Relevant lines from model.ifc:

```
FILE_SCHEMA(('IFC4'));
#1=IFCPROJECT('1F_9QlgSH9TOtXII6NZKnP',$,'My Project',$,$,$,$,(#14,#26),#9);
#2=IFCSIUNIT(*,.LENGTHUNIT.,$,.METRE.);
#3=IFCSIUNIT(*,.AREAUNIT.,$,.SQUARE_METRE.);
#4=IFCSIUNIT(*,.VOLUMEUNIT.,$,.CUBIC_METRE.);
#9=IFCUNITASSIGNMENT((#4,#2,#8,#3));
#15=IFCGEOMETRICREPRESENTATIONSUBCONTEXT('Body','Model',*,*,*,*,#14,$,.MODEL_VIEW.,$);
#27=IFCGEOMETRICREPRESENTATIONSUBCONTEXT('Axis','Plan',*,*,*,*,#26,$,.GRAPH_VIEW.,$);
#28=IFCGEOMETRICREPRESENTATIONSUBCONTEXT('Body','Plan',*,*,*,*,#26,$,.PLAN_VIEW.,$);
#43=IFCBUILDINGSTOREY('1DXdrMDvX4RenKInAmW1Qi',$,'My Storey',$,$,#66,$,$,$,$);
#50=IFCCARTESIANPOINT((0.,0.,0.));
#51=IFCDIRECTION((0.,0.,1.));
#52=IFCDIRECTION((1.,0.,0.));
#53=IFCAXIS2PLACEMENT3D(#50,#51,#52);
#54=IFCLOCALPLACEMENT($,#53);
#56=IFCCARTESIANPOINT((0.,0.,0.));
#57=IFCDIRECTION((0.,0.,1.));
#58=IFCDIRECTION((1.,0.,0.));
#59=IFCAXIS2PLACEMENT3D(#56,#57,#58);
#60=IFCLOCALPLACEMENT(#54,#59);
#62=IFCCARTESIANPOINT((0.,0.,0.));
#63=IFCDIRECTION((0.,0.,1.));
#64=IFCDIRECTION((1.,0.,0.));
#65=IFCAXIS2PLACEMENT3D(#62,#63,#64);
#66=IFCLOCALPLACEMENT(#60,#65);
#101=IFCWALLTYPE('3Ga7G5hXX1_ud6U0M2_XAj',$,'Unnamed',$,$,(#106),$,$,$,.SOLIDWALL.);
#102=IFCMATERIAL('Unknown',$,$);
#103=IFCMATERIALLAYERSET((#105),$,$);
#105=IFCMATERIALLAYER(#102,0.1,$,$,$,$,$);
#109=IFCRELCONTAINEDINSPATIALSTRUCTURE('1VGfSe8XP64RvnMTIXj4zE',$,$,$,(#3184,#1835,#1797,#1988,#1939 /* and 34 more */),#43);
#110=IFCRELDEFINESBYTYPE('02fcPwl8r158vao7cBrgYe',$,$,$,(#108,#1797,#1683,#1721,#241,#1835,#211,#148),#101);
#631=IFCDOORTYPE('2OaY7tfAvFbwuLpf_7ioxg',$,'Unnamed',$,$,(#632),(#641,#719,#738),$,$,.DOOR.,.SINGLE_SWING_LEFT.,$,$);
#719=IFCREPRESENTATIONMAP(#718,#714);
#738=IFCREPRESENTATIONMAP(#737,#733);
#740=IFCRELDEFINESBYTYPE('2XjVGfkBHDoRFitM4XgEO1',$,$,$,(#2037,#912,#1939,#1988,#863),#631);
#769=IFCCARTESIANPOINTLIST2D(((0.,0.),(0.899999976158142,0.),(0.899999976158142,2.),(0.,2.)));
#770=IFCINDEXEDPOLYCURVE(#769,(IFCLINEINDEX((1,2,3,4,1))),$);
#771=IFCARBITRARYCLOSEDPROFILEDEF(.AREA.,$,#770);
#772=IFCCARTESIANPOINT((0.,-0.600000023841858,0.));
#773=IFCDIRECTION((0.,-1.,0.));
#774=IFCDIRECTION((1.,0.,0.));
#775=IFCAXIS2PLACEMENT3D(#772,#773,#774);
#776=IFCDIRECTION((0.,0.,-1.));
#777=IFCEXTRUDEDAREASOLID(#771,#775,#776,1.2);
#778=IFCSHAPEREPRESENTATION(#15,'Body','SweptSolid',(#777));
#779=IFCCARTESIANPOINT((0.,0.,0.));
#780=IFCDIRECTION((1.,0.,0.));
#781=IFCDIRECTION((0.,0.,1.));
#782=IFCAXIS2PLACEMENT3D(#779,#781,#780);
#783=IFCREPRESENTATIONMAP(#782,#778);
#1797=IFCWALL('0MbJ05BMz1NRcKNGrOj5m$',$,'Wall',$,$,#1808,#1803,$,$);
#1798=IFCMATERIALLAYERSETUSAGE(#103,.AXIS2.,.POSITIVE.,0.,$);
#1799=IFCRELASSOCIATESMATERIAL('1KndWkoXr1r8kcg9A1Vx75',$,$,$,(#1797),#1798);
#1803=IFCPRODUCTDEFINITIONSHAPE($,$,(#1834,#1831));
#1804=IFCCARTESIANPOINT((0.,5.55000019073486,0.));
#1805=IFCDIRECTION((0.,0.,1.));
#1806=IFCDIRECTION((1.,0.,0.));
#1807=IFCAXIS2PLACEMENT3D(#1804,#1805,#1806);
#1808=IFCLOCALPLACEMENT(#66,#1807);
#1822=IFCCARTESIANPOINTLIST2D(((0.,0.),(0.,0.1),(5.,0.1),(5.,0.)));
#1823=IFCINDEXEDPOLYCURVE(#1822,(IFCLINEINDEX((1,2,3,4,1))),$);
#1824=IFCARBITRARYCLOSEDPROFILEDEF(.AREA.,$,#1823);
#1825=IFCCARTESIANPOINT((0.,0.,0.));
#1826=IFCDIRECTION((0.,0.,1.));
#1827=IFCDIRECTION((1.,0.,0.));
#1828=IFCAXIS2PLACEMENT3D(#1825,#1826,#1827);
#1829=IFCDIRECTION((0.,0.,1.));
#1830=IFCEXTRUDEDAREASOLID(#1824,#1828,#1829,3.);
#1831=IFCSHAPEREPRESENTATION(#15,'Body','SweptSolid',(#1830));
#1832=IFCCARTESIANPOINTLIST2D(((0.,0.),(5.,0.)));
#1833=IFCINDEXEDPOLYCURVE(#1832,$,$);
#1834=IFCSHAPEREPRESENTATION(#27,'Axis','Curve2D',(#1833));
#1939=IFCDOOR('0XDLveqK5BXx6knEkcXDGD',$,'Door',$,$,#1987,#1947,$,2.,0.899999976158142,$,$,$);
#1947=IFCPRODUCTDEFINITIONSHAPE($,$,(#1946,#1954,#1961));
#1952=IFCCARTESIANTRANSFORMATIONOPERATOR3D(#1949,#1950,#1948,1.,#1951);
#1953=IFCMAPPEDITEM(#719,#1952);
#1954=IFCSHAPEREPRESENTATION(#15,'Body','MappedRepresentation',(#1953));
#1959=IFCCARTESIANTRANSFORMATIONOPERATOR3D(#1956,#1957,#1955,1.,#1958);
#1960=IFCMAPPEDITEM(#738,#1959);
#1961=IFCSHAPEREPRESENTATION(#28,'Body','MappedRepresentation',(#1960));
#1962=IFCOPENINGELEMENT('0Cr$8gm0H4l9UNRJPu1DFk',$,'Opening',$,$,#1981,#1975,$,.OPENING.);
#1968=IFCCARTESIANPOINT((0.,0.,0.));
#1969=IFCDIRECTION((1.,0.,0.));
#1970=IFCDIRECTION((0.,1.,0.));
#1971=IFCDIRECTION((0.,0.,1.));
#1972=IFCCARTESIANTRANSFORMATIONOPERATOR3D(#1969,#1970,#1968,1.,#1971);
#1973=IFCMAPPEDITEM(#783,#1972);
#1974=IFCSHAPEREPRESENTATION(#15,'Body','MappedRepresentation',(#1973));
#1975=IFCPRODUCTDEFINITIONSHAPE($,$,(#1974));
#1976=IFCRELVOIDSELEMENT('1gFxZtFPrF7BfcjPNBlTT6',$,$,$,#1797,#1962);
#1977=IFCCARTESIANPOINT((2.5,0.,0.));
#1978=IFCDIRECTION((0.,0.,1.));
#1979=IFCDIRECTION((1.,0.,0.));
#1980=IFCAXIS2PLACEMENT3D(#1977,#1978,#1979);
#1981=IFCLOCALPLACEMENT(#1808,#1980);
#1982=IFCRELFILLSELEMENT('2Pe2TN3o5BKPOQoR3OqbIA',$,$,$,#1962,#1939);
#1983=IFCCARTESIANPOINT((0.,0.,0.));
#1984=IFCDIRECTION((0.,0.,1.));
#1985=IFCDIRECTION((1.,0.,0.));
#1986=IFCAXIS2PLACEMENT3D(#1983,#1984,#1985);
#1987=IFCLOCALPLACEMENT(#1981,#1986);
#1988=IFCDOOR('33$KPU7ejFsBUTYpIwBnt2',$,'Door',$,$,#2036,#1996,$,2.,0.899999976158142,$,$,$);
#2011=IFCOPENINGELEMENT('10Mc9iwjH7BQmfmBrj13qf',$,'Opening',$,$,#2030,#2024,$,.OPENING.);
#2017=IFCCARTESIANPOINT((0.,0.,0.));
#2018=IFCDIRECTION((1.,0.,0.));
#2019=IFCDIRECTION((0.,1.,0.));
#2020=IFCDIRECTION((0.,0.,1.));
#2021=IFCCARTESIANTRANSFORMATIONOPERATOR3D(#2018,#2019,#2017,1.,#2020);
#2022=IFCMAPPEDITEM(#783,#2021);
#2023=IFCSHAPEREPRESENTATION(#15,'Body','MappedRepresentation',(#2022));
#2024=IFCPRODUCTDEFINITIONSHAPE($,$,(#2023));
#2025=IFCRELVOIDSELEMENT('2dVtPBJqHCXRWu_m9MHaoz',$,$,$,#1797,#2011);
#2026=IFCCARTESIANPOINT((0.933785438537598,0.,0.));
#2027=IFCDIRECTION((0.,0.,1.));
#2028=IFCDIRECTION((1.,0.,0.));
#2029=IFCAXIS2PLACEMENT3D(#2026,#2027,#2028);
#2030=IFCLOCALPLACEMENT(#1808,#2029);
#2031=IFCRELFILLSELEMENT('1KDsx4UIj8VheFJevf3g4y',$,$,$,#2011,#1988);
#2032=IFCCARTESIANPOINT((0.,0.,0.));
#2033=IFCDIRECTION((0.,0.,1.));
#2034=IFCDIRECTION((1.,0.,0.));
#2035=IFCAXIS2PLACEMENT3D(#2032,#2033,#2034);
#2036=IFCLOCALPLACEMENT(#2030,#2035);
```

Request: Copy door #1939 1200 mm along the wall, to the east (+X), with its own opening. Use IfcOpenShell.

```python
import ifcopenshell
import ifcopenshell.api.feature
import ifcopenshell.api.geometry
import ifcopenshell.api.root
import ifcopenshell.geom
import ifcopenshell.util.element
import ifcopenshell.util.placement
import ifcopenshell.util.shape
import ifcopenshell.util.unit

model = ifcopenshell.open("model.ifc")
unit_scale = ifcopenshell.util.unit.calculate_unit_scale(model)
settings = ifcopenshell.geom.settings()


def volume(element):
    """Net volume in cubic metres, openings subtracted."""
    shape = ifcopenshell.geom.create_shape(settings, element)
    return ifcopenshell.util.shape.get_volume(shape.geometry)


door = model.by_guid("0XDLveqK5BXx6knEkcXDGD")
opening = door.FillsVoids[0].RelatingOpeningElement
wall = opening.VoidsElements[0].RelatingBuildingElement
before = volume(wall)
shift = ifcopenshell.util.placement.get_local_placement(wall.ObjectPlacement)[:3, 0] * 1.2 / unit_scale

# copy_class copies the void relationship, type, container and properties, but no geometry.
new_opening = ifcopenshell.api.root.copy_class(model, product=opening)
new_opening.Representation = ifcopenshell.util.element.copy_deep(
    model, opening.Representation, exclude=["IfcGeometricRepresentationContext", "IfcRepresentationMap"]
)
new_door = ifcopenshell.api.root.copy_class(model, product=door)
new_door.Representation = ifcopenshell.util.element.copy_deep(
    model, door.Representation, exclude=["IfcGeometricRepresentationContext", "IfcRepresentationMap"]
)
ifcopenshell.api.feature.add_filling(model, opening=new_opening, element=new_door)

for old, new in ((opening, new_opening), (door, new_door)):
    matrix = ifcopenshell.util.placement.get_local_placement(old.ObjectPlacement)
    matrix[:3, 3] += shift
    ifcopenshell.api.geometry.edit_object_placement(model, product=new, matrix=matrix, is_si=False)

after = volume(wall)

print(f"wall volume {before:.3f} -> {after:.3f} m3")

model.write("model_v2.ifc")
```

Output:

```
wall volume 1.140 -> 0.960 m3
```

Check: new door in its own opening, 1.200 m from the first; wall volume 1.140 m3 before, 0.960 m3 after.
